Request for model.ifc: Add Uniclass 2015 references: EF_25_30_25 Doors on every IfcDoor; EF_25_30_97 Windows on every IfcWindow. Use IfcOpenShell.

First a look at what the model holds.

```python
import ifcopenshell

model = ifcopenshell.open("model.ifc")
print(model.schema)
print("classifications:", [c.Name for c in model.by_type("IfcClassification")])
for ifc_class in ("IfcDoor", "IfcRoof", "IfcStair", "IfcWall", "IfcWindow"):
    print(ifc_class, len(model.by_type(ifc_class)))
```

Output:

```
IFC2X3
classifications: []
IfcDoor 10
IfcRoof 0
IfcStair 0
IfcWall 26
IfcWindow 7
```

```python
import ifcopenshell
import ifcopenshell.api.classification

model = ifcopenshell.open("model.ifc")

# IFC2X3 requires Source and Edition and has no link from the project to the system.
system = model.create_entity("IfcClassification", Source="NBS", Edition="2015", Name="Uniclass 2015")

codes = {
    "IfcDoor": ("EF_25_30_25", "Doors"),
    "IfcWindow": ("EF_25_30_97", "Windows"),
}
for ifc_class, (code, name) in codes.items():
    products = model.by_type(ifc_class)
    ifcopenshell.api.classification.add_reference(
        model, products=products, classification=system, identification=code, name=name
    )
    print(code, len(products))

model.write("model_v2.ifc")
```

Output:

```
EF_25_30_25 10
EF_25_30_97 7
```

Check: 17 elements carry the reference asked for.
